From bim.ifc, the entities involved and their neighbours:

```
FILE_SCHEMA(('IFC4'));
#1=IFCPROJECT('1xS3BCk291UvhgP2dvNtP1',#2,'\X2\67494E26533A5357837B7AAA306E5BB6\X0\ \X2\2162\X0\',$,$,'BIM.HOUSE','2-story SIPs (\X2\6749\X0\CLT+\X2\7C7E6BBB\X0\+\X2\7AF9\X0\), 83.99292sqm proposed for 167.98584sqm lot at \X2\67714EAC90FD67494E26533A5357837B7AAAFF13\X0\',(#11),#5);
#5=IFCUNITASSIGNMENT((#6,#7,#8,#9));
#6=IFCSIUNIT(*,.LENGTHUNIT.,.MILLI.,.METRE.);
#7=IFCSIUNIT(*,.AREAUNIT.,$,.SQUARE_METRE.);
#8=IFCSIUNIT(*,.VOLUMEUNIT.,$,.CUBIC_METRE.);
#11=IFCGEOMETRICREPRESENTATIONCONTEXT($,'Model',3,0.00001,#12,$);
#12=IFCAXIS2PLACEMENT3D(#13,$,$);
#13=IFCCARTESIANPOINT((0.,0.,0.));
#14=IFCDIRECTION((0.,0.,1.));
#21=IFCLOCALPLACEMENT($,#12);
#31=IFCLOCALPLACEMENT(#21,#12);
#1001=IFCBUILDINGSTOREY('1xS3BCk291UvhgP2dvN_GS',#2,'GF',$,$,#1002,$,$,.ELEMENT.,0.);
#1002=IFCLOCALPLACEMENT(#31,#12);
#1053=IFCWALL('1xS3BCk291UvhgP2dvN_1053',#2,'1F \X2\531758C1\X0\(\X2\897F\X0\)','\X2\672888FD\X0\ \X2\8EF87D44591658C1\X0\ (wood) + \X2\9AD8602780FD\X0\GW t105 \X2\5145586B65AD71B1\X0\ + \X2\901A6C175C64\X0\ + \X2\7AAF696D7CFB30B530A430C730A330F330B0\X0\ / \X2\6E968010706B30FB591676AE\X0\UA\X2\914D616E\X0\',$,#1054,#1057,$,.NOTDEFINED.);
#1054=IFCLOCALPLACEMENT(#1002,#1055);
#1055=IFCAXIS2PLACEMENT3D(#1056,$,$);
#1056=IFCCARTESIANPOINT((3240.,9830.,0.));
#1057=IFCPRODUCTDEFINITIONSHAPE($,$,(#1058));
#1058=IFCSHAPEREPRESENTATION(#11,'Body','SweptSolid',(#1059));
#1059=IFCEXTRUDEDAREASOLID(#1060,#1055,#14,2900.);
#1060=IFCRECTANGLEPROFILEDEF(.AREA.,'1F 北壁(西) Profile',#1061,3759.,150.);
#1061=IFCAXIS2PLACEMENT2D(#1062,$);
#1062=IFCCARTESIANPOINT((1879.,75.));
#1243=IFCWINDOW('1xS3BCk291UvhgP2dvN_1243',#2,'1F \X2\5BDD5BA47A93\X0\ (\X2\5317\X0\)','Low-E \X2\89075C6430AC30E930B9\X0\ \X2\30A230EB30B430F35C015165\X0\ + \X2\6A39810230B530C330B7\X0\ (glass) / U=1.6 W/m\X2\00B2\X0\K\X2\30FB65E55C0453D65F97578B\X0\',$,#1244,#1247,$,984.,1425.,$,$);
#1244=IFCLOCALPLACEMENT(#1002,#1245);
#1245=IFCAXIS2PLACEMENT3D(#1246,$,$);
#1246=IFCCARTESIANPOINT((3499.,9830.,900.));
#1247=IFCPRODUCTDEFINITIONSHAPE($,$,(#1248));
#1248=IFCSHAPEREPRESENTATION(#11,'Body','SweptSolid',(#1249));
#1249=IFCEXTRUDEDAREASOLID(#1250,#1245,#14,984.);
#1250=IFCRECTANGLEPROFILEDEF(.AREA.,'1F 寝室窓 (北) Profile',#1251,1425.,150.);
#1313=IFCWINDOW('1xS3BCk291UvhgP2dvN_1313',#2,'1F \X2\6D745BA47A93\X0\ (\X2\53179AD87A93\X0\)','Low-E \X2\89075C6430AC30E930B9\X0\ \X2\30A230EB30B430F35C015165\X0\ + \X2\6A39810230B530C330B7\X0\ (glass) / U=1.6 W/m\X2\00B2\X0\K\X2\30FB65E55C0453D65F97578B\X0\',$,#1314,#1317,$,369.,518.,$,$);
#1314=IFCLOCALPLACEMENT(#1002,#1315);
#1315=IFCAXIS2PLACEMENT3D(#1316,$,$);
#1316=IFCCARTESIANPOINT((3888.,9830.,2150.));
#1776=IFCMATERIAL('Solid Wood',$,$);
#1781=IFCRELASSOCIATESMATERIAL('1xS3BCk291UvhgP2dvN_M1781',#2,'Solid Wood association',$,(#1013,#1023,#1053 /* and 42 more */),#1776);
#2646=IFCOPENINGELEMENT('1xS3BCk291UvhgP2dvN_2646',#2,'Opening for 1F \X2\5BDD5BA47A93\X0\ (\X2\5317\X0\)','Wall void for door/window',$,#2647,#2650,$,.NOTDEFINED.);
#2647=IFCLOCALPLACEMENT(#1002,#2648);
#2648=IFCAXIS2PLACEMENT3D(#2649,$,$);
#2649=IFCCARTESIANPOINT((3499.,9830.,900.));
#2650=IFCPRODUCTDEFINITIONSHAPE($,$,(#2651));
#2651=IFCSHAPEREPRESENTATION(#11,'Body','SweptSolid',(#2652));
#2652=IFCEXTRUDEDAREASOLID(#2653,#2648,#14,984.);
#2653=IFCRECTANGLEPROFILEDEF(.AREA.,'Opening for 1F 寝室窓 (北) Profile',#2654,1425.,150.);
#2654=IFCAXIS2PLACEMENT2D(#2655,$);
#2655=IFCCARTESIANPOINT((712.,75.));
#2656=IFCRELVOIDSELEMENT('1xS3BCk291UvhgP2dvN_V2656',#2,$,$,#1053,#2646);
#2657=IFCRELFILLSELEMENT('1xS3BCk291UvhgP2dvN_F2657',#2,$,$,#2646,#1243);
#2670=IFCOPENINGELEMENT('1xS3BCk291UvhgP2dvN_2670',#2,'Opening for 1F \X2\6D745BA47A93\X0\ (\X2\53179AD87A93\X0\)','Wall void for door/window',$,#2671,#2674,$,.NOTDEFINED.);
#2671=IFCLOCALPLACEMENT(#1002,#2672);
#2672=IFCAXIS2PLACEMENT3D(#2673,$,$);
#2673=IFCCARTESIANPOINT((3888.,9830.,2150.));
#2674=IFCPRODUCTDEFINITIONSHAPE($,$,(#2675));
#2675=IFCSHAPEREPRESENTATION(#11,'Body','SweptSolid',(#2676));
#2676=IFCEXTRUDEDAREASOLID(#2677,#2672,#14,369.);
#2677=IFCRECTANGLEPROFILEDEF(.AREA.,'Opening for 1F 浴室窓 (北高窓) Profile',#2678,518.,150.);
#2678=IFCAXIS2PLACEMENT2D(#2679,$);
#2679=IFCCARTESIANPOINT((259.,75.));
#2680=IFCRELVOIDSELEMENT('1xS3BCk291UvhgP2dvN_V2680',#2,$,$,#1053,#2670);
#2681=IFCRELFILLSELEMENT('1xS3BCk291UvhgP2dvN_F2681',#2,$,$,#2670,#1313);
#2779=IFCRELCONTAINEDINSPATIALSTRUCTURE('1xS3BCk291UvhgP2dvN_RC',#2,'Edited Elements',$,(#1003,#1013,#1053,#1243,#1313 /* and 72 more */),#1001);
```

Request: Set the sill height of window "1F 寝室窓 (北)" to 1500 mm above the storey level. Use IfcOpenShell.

```python
import numpy as np
import ifcopenshell
import ifcopenshell.api.geometry
import ifcopenshell.geom
import ifcopenshell.util.element
import ifcopenshell.util.placement
import ifcopenshell.util.shape
import ifcopenshell.util.unit

model = ifcopenshell.open("bim.ifc")
unit_scale = ifcopenshell.util.unit.calculate_unit_scale(model)

window = model.by_id(1243)
opening = window.FillsVoids[0].RelatingOpeningElement
storey = ifcopenshell.util.element.get_container(window, ifc_class="IfcBuildingStorey")
level = ifcopenshell.util.placement.get_local_placement(storey.ObjectPlacement)[2, 3]

# The opening's origin need not be at the sill, so measure its lowest point.
shape = ifcopenshell.geom.create_shape(ifcopenshell.geom.settings(), opening)
bottom = ifcopenshell.util.shape.get_shape_bottom_elevation(shape, shape.geometry) / unit_scale
dz = level + 1.5 / unit_scale - bottom

shift = np.array([0.0, 0.0, dz])
# The window is not placed relative to its opening, so move both.
for product in (opening, window):
    matrix = ifcopenshell.util.placement.get_local_placement(product.ObjectPlacement)
    matrix[:3, 3] += shift
    ifcopenshell.api.geometry.edit_object_placement(model, product=product, matrix=matrix, is_si=False)

print(f"moved by {dz * unit_scale:+.3f} m")

model.write("bim_v2.ifc")
```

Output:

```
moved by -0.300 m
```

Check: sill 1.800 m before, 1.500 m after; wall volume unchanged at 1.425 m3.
